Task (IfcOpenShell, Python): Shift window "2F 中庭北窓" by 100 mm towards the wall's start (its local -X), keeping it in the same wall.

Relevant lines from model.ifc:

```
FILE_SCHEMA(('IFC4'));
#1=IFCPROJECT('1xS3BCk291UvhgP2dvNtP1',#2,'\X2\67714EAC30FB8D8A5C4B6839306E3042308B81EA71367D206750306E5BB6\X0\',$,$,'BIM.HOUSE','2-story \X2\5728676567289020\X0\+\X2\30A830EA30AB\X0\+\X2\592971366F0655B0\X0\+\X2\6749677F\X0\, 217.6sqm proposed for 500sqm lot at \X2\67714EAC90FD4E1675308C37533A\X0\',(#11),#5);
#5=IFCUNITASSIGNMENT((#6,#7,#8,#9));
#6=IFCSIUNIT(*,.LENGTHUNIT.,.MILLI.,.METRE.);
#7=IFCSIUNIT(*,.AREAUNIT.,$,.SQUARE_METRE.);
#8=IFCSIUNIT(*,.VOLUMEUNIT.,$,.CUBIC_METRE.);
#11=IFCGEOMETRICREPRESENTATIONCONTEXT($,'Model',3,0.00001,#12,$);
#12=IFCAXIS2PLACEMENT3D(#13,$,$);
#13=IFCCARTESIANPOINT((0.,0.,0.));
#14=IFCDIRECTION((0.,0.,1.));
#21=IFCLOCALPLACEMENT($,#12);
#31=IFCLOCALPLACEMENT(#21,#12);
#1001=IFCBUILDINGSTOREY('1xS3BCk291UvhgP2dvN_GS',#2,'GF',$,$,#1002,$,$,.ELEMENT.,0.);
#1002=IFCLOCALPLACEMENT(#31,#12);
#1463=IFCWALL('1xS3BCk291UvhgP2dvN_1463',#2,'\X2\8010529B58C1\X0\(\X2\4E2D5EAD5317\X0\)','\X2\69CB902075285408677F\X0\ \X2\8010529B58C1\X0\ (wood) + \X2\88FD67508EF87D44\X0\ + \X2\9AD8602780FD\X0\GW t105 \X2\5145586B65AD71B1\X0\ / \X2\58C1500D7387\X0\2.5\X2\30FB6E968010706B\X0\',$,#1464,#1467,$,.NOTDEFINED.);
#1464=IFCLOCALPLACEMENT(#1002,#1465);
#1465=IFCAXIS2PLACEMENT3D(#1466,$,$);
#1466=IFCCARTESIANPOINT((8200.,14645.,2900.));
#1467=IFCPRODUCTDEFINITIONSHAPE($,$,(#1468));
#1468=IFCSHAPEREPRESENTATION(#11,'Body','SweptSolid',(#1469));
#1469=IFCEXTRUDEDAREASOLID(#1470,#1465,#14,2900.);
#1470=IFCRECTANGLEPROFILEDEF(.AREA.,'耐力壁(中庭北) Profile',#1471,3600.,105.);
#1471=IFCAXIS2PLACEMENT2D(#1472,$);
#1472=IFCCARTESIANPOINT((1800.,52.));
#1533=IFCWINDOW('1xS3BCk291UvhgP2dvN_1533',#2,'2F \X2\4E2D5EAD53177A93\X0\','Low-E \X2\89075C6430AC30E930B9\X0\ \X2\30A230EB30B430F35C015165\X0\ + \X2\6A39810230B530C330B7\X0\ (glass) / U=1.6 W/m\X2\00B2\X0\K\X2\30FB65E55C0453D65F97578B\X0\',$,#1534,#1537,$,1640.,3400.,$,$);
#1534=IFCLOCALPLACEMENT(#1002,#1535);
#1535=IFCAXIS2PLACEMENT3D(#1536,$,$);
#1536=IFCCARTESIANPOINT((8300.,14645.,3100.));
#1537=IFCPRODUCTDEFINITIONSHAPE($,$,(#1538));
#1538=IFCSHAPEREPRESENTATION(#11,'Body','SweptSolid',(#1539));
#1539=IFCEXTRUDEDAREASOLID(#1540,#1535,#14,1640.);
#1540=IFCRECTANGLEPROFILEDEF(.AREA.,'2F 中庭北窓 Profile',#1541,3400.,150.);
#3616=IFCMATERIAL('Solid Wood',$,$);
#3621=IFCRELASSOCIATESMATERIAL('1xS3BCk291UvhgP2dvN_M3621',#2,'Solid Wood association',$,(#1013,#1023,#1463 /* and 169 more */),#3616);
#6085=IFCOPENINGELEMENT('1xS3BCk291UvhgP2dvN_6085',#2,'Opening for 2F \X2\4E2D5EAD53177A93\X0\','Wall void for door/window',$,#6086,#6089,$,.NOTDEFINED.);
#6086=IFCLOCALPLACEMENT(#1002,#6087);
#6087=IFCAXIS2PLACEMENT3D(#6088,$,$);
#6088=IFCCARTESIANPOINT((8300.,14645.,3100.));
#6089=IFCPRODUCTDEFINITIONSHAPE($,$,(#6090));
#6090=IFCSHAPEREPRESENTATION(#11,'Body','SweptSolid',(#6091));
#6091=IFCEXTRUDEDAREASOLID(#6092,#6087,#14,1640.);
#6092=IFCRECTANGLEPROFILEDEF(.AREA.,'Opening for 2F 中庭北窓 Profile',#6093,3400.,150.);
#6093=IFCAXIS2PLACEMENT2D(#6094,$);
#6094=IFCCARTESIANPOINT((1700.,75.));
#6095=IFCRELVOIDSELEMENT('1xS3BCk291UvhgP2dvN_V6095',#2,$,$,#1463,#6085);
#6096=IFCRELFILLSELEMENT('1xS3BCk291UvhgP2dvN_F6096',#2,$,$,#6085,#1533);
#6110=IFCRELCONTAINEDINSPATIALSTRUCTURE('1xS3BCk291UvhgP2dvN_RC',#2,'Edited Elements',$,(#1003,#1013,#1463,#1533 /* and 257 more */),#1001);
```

```python
import ifcopenshell
import ifcopenshell.api.geometry
import ifcopenshell.util.placement
import ifcopenshell.util.unit

model = ifcopenshell.open("model.ifc")
unit_scale = ifcopenshell.util.unit.calculate_unit_scale(model)

window = model.by_guid("1xS3BCk291UvhgP2dvN_1533")
opening = window.FillsVoids[0].RelatingOpeningElement
wall = opening.VoidsElements[0].RelatingBuildingElement

wall_matrix = ifcopenshell.util.placement.get_local_placement(wall.ObjectPlacement)
shift = wall_matrix[:3, 0] * -0.1 / unit_scale
before = ifcopenshell.util.placement.get_local_placement(window.ObjectPlacement)[:3, 3].copy()

# The window is not placed relative to its opening, so move both.
for product in (opening, window):
    matrix = ifcopenshell.util.placement.get_local_placement(product.ObjectPlacement)
    matrix[:3, 3] += shift
    ifcopenshell.api.geometry.edit_object_placement(model, product=product, matrix=matrix, is_si=False)

after = ifcopenshell.util.placement.get_local_placement(window.ObjectPlacement)[:3, 3]
print("window moved by", (after - before).round(3) + 0.0)

model.write("model-out.ifc")
```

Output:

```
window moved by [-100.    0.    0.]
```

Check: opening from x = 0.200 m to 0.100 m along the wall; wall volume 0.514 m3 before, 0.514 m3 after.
